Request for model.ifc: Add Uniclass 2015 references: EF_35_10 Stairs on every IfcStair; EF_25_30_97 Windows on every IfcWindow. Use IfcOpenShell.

First a look at what the model holds.

```python
import ifcopenshell

model = ifcopenshell.open("model.ifc")
print(model.schema)
print("classifications:", [c.Name for c in model.by_type("IfcClassification")])
for ifc_class in ("IfcDoor", "IfcRoof", "IfcStair", "IfcWall", "IfcWindow"):
    print(ifc_class, len(model.by_type(ifc_class)))
```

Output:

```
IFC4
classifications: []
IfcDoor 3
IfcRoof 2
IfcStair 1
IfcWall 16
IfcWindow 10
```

```python
import ifcopenshell
import ifcopenshell.api.classification

model = ifcopenshell.open("model.ifc")

system = ifcopenshell.api.classification.add_classification(model, classification="Uniclass 2015")

codes = {
    "IfcStair": ("EF_35_10", "Stairs"),
    "IfcWindow": ("EF_25_30_97", "Windows"),
}
for ifc_class, (code, name) in codes.items():
    products = model.by_type(ifc_class)
    ifcopenshell.api.classification.add_reference(
        model, products=products, classification=system, identification=code, name=name
    )
    print(code, len(products))

model.write("model_edited.ifc")
```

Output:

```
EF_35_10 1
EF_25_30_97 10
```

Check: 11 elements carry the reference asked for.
